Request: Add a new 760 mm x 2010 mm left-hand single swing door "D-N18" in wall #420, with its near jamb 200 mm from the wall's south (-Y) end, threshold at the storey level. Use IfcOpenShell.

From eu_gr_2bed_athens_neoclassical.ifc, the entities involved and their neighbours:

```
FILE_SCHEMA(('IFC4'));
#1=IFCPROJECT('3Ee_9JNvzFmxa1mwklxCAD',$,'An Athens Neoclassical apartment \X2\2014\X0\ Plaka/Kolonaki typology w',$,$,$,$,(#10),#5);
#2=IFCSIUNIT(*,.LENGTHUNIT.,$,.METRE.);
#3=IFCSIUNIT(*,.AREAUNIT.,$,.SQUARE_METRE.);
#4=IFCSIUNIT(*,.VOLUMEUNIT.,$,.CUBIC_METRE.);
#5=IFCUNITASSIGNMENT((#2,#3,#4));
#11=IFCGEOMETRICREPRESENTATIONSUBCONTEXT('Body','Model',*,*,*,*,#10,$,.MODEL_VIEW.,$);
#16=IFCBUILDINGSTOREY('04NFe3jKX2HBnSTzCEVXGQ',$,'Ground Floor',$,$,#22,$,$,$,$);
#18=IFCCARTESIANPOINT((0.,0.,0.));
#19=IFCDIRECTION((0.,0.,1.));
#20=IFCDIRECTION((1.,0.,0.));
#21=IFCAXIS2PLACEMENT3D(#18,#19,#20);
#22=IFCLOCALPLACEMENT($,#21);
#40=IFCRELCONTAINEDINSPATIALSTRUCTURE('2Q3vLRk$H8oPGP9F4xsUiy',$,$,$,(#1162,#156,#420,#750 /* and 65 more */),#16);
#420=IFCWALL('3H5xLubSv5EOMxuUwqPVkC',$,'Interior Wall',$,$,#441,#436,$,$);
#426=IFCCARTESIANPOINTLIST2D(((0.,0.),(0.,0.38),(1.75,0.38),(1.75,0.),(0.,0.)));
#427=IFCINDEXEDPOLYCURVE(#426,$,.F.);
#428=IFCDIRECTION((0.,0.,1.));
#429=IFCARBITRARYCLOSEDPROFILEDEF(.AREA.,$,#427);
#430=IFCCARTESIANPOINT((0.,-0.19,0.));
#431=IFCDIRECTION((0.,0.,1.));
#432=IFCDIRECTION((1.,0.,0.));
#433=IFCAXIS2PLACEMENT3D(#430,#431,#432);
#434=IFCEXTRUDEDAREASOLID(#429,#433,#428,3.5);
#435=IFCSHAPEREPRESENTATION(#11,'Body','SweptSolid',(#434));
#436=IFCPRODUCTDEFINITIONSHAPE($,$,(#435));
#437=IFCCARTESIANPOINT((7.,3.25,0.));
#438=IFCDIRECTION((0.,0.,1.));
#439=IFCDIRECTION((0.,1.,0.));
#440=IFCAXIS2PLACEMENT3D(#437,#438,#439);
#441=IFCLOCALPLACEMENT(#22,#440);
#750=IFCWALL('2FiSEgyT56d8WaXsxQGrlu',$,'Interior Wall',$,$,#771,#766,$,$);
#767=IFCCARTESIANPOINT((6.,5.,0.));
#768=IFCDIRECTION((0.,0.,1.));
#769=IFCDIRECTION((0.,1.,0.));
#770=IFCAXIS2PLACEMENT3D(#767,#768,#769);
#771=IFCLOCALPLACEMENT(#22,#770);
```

```python
import numpy as np
import ifcopenshell
import ifcopenshell.api.feature
import ifcopenshell.api.geometry
import ifcopenshell.api.root
import ifcopenshell.api.spatial
import ifcopenshell.geom
import ifcopenshell.util.element
import ifcopenshell.util.placement
import ifcopenshell.util.representation
import ifcopenshell.util.shape
import ifcopenshell.util.unit

model = ifcopenshell.open("eu_gr_2bed_athens_neoclassical.ifc")
unit_scale = ifcopenshell.util.unit.calculate_unit_scale(model)
settings = ifcopenshell.geom.settings()


def volume(element):
    """Net volume in cubic metres, openings subtracted."""
    shape = ifcopenshell.geom.create_shape(settings, element)
    return ifcopenshell.util.shape.get_volume(shape.geometry)


wall = model.by_guid("3H5xLubSv5EOMxuUwqPVkC")
storey = ifcopenshell.util.element.get_container(wall, ifc_class="IfcBuildingStorey")
context = ifcopenshell.util.representation.get_context(model, "Model", "Body", "MODEL_VIEW")
before = volume(wall)

width, height, from_end, sill = 0.76, 2.01, 0.2, 0.0  # metres

# The wall runs along its own X axis, and the end named is its -X end.
wall_shape = ifcopenshell.geom.create_shape(settings, wall)
x, y, z = ifcopenshell.util.shape.get_vertices(wall_shape.geometry).T
start = x.min() + from_end
face, thickness = float(y.min()), float(y.max() - y.min())
wall_matrix = ifcopenshell.util.placement.get_local_placement(wall.ObjectPlacement)
level = ifcopenshell.util.placement.get_local_placement(storey.ObjectPlacement)[2, 3]


def in_wall(x, y):
    """Placement at x, y metres in the wall's axes, at sill height."""
    matrix = wall_matrix.copy()
    matrix[:, 3] = wall_matrix @ np.array([x / unit_scale, y / unit_scale, 0.0, 1.0])
    matrix[2, 3] = level + sill / unit_scale
    return matrix


# Opening: a box that overshoots both wall faces by 50 mm.
opening = ifcopenshell.api.root.create_entity(model, ifc_class="IfcOpeningElement", predefined_type="OPENING")
box = ifcopenshell.api.geometry.add_wall_representation(
    model, context=context, length=width, height=height, thickness=thickness + 0.1
)
ifcopenshell.api.geometry.assign_representation(model, product=opening, representation=box)
ifcopenshell.api.geometry.edit_object_placement(model, product=opening, matrix=in_wall(start, face - 0.05), is_si=False)
ifcopenshell.api.feature.add_feature(model, feature=opening, element=wall)

door = ifcopenshell.api.root.create_entity(model, ifc_class="IfcDoor", name="D-N18", predefined_type="DOOR")
door.OverallWidth, door.OverallHeight = width / unit_scale, height / unit_scale
door.OperationType = "SINGLE_SWING_LEFT"
body = ifcopenshell.api.geometry.add_door_representation(
    model,
    context=context,
    overall_width=door.OverallWidth,
    overall_height=door.OverallHeight,
    operation_type="SINGLE_SWING_LEFT",
    lining_properties={"LiningDepth": thickness / unit_scale, "ThresholdDepth": thickness / unit_scale},
)
ifcopenshell.api.geometry.assign_representation(model, product=door, representation=body)
ifcopenshell.api.spatial.assign_container(model, products=[door], relating_structure=storey)
ifcopenshell.api.feature.add_filling(model, opening=opening, element=door)

# The lining spans the wall, so the door starts at the wall face.
ifcopenshell.api.geometry.edit_object_placement(model, product=door, matrix=in_wall(start, face), is_si=False)

after = volume(wall)

print(f"wall volume {before:.3f} -> {after:.3f} m3")

model.write("eu_gr_2bed_athens_neoclassical_rev.ifc")
```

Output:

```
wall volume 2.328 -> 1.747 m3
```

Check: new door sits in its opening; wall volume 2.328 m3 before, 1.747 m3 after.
